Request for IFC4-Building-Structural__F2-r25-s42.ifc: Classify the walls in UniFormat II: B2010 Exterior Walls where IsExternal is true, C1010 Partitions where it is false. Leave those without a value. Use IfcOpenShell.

First a look at what the model holds.

```python
import ifcopenshell
import ifcopenshell.util.element

model = ifcopenshell.open("IFC4-Building-Structural__F2-r25-s42.ifc")
print(model.schema)
print("classifications:", [c.Name for c in model.by_type("IfcClassification")])
values = [ifcopenshell.util.element.get_pset(e, "Pset_WallCommon", "IsExternal") for e in model.by_type("IfcWall")]
for value in (True, False, None):
    print("IsExternal", value, values.count(value))
```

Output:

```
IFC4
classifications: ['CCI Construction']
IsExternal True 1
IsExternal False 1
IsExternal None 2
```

```python
import ifcopenshell
import ifcopenshell.api.classification
import ifcopenshell.util.element

model = ifcopenshell.open("IFC4-Building-Structural__F2-r25-s42.ifc")

system = ifcopenshell.api.classification.add_classification(model, classification="UniFormat II")

walls = model.by_type("IfcWall")
external = {e: ifcopenshell.util.element.get_pset(e, "Pset_WallCommon", "IsExternal") for e in walls}
for flag, code, name in ((True, "B2010", "Exterior Walls"), (False, "C1010", "Partitions")):
    products = [e for e in walls if external[e] is flag]
    ifcopenshell.api.classification.add_reference(
        model, products=products, classification=system, identification=code, name=name
    )
    print(code, len(products))

model.write("IFC4-Building-Structural__F2-r25-s42_edited.ifc")
```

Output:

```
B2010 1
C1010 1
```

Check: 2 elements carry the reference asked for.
